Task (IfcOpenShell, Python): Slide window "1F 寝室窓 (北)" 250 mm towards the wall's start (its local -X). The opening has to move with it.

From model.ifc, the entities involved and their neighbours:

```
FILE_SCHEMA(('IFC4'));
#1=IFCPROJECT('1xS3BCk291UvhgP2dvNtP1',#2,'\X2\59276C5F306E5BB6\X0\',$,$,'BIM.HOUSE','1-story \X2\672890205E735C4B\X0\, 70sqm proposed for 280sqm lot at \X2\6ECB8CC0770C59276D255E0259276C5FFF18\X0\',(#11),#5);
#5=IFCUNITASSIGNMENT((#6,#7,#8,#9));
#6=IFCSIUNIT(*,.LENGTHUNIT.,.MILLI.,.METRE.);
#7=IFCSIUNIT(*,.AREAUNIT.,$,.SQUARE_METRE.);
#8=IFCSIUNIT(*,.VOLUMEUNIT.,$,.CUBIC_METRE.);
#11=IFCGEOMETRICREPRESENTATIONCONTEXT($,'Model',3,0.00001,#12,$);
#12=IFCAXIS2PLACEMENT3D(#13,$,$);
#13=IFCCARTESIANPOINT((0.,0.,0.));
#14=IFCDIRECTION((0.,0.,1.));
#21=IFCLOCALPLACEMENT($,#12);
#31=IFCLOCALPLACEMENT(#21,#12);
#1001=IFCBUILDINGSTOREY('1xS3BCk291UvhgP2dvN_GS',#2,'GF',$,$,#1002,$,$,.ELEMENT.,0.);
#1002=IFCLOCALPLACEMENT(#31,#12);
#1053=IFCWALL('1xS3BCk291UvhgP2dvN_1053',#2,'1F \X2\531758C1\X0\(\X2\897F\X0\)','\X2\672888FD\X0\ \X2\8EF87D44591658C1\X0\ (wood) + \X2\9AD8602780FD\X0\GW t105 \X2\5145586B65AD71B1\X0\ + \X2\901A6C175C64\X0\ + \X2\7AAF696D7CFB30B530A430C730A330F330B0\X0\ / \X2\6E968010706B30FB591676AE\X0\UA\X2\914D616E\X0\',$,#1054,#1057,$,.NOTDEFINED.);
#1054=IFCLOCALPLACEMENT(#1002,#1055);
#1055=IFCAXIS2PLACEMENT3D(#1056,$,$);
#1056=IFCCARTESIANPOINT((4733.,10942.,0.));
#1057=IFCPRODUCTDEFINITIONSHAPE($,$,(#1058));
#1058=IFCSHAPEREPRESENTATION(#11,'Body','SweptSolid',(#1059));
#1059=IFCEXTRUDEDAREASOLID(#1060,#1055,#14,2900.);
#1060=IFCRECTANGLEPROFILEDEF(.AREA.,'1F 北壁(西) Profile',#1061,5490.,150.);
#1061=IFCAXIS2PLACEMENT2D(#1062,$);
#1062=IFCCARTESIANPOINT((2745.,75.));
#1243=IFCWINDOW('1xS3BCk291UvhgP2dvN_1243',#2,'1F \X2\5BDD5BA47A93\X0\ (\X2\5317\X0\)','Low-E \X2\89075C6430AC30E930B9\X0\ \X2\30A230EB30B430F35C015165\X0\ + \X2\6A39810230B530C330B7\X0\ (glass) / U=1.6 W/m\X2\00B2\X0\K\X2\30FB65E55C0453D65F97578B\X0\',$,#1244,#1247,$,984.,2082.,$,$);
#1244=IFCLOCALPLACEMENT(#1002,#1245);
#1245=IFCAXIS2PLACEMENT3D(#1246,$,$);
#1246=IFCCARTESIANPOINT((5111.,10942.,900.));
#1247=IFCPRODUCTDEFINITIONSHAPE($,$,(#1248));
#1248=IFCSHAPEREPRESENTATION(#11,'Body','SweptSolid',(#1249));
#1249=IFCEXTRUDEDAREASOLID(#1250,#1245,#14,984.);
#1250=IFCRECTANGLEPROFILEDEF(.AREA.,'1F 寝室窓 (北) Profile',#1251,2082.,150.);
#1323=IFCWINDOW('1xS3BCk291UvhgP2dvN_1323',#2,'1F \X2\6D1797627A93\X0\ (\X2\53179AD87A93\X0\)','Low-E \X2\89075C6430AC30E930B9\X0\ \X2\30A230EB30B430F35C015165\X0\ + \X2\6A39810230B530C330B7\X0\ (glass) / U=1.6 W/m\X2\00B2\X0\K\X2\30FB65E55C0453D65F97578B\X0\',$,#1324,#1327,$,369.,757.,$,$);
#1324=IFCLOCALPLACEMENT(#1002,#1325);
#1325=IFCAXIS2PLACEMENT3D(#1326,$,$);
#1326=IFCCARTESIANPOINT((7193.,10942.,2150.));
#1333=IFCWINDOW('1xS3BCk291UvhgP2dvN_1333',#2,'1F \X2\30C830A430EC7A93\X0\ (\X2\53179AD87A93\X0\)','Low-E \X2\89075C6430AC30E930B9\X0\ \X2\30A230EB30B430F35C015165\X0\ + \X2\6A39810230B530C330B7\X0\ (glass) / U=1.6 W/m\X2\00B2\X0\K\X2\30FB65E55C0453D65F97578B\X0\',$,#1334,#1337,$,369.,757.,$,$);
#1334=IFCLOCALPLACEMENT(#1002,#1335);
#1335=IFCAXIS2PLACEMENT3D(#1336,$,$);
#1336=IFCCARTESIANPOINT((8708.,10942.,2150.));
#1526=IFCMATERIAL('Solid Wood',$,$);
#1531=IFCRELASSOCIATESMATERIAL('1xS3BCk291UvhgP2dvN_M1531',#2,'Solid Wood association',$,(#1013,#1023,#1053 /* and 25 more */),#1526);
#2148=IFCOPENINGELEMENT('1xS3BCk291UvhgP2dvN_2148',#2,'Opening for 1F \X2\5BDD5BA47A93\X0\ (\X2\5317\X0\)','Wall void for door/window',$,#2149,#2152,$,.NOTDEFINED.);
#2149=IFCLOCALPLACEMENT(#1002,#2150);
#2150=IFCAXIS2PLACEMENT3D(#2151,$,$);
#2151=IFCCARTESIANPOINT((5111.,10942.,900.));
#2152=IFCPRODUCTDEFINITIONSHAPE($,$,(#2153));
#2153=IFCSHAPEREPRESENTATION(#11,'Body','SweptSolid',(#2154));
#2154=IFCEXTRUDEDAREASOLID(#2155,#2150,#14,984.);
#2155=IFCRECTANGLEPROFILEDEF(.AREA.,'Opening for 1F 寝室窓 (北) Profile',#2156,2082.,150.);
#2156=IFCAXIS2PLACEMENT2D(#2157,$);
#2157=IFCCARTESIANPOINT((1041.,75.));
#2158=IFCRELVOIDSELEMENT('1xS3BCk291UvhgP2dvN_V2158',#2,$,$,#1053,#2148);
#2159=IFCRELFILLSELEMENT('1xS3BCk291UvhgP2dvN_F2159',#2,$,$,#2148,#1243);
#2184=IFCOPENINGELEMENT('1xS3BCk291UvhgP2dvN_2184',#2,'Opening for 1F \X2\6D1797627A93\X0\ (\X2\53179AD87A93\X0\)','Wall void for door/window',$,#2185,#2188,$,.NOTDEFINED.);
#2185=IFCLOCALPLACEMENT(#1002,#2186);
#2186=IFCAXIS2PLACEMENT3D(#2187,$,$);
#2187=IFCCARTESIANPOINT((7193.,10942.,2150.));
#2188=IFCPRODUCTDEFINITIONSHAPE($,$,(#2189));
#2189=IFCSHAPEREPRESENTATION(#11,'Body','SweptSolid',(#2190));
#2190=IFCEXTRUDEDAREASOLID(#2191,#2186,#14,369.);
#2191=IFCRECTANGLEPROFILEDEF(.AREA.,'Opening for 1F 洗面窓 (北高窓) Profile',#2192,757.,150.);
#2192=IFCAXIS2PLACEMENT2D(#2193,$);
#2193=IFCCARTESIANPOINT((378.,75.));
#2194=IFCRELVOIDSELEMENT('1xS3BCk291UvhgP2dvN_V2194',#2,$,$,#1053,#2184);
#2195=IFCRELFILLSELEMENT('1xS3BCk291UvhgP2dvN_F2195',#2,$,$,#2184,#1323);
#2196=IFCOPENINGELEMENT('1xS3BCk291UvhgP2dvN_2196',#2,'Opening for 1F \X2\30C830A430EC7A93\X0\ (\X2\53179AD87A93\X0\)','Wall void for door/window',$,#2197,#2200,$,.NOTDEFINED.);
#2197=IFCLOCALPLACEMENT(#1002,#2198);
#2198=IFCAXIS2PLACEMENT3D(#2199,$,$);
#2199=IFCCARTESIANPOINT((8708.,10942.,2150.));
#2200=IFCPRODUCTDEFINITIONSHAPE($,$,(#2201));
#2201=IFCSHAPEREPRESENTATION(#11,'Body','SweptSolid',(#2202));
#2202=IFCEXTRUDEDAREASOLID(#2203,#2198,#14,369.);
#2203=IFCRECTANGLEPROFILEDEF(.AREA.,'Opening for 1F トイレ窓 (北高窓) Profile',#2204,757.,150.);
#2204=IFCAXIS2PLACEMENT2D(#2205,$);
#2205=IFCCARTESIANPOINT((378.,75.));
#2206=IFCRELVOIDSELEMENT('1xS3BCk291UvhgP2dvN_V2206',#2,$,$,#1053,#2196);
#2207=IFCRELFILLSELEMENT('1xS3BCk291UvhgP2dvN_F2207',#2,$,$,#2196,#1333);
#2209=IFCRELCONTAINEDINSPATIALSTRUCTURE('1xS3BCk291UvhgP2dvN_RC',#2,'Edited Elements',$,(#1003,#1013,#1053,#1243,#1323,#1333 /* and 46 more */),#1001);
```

```python
import ifcopenshell
import ifcopenshell.api.geometry
import ifcopenshell.util.placement

model = ifcopenshell.open("model.ifc")

window = model.by_guid("1xS3BCk291UvhgP2dvN_1243")
opening = window.FillsVoids[0].RelatingOpeningElement
wall = opening.VoidsElements[0].RelatingBuildingElement

wall_matrix = ifcopenshell.util.placement.get_local_placement(wall.ObjectPlacement)
shift = wall_matrix[:3, 0] * -250.0
before = ifcopenshell.util.placement.get_local_placement(window.ObjectPlacement)[:3, 3].copy()

# The window is not placed relative to its opening, so move both.
for product in (opening, window):
    matrix = ifcopenshell.util.placement.get_local_placement(product.ObjectPlacement)
    matrix[:3, 3] += shift
    ifcopenshell.api.geometry.edit_object_placement(model, product=product, matrix=matrix, is_si=False)

after = ifcopenshell.util.placement.get_local_placement(window.ObjectPlacement)[:3, 3]
print("window moved by", (after - before).round(3) + 0.0)

model.write("model_v2.ifc")
```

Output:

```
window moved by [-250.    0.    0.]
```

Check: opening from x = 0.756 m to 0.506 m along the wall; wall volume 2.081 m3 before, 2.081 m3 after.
